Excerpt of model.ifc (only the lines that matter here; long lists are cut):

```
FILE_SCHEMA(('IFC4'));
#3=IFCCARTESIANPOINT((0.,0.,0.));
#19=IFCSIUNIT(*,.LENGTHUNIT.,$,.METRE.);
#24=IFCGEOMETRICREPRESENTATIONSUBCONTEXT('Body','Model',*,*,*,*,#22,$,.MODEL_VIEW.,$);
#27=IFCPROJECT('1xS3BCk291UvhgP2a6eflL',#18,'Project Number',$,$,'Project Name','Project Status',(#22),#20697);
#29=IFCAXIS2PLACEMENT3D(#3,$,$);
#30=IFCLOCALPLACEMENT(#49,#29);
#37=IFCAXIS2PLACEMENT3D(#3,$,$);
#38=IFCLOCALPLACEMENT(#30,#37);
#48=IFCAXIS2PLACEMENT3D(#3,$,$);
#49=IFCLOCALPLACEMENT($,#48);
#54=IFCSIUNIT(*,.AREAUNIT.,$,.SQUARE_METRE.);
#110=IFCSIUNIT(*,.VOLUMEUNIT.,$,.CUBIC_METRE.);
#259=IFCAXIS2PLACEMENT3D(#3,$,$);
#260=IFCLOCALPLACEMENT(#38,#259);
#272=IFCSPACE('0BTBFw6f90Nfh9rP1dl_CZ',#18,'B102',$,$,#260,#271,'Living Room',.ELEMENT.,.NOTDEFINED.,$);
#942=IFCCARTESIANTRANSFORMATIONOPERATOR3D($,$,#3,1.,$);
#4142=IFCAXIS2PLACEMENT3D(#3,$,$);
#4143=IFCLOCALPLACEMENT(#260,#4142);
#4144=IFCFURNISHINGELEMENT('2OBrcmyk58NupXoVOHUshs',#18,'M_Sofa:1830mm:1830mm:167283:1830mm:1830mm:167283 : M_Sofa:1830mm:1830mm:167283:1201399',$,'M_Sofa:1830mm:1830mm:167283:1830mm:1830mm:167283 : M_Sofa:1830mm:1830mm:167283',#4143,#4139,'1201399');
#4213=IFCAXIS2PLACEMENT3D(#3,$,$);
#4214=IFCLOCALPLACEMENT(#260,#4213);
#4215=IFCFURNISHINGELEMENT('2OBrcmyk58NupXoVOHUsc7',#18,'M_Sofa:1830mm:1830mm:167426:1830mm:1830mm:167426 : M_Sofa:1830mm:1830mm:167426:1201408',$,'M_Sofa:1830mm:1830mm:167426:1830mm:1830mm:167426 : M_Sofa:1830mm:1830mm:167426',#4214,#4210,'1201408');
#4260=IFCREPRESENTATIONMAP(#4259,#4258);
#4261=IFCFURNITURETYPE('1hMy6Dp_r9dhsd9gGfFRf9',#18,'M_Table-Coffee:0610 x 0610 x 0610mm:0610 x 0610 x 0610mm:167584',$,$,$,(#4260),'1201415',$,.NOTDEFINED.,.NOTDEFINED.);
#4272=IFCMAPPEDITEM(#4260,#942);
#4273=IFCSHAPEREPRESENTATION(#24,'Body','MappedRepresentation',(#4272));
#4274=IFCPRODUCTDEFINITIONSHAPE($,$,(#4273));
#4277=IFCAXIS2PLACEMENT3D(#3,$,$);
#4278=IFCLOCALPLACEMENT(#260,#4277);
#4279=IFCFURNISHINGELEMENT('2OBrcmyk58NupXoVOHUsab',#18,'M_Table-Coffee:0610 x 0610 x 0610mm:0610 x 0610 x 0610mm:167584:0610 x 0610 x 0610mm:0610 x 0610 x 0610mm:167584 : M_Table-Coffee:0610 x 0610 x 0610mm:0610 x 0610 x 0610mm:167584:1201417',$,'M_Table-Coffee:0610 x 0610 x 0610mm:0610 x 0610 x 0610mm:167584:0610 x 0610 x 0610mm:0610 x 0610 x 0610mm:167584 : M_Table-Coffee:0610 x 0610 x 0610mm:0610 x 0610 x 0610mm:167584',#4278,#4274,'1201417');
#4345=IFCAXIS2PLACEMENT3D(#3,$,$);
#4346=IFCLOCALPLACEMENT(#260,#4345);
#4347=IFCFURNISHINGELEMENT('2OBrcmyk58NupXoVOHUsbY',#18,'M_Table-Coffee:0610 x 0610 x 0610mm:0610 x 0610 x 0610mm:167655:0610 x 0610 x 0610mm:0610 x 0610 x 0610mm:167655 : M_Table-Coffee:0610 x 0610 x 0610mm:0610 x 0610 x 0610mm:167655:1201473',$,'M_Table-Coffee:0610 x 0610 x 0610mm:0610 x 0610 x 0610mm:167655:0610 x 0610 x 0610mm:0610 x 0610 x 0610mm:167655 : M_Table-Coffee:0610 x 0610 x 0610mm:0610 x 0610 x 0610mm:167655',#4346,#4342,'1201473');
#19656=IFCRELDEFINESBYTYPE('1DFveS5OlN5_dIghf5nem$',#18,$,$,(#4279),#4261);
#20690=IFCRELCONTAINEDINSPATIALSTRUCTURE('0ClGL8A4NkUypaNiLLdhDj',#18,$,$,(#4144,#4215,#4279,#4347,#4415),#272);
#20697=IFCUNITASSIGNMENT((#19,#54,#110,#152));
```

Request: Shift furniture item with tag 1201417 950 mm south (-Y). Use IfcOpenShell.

```python
import ifcopenshell
import ifcopenshell.api.geometry
import ifcopenshell.util.placement

model = ifcopenshell.open("model.ifc")

item = model.by_guid("2OBrcmyk58NupXoVOHUsab")
matrix = ifcopenshell.util.placement.get_local_placement(item.ObjectPlacement)
matrix[1, 3] -= 0.95
ifcopenshell.api.geometry.edit_object_placement(model, product=item, matrix=matrix, is_si=False)

print(ifcopenshell.util.placement.get_local_placement(item.ObjectPlacement).round(3) + 0.0)

model.write("model-out.ifc")
```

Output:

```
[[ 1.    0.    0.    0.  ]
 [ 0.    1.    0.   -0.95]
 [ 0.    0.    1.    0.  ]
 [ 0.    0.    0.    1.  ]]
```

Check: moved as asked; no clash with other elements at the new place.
